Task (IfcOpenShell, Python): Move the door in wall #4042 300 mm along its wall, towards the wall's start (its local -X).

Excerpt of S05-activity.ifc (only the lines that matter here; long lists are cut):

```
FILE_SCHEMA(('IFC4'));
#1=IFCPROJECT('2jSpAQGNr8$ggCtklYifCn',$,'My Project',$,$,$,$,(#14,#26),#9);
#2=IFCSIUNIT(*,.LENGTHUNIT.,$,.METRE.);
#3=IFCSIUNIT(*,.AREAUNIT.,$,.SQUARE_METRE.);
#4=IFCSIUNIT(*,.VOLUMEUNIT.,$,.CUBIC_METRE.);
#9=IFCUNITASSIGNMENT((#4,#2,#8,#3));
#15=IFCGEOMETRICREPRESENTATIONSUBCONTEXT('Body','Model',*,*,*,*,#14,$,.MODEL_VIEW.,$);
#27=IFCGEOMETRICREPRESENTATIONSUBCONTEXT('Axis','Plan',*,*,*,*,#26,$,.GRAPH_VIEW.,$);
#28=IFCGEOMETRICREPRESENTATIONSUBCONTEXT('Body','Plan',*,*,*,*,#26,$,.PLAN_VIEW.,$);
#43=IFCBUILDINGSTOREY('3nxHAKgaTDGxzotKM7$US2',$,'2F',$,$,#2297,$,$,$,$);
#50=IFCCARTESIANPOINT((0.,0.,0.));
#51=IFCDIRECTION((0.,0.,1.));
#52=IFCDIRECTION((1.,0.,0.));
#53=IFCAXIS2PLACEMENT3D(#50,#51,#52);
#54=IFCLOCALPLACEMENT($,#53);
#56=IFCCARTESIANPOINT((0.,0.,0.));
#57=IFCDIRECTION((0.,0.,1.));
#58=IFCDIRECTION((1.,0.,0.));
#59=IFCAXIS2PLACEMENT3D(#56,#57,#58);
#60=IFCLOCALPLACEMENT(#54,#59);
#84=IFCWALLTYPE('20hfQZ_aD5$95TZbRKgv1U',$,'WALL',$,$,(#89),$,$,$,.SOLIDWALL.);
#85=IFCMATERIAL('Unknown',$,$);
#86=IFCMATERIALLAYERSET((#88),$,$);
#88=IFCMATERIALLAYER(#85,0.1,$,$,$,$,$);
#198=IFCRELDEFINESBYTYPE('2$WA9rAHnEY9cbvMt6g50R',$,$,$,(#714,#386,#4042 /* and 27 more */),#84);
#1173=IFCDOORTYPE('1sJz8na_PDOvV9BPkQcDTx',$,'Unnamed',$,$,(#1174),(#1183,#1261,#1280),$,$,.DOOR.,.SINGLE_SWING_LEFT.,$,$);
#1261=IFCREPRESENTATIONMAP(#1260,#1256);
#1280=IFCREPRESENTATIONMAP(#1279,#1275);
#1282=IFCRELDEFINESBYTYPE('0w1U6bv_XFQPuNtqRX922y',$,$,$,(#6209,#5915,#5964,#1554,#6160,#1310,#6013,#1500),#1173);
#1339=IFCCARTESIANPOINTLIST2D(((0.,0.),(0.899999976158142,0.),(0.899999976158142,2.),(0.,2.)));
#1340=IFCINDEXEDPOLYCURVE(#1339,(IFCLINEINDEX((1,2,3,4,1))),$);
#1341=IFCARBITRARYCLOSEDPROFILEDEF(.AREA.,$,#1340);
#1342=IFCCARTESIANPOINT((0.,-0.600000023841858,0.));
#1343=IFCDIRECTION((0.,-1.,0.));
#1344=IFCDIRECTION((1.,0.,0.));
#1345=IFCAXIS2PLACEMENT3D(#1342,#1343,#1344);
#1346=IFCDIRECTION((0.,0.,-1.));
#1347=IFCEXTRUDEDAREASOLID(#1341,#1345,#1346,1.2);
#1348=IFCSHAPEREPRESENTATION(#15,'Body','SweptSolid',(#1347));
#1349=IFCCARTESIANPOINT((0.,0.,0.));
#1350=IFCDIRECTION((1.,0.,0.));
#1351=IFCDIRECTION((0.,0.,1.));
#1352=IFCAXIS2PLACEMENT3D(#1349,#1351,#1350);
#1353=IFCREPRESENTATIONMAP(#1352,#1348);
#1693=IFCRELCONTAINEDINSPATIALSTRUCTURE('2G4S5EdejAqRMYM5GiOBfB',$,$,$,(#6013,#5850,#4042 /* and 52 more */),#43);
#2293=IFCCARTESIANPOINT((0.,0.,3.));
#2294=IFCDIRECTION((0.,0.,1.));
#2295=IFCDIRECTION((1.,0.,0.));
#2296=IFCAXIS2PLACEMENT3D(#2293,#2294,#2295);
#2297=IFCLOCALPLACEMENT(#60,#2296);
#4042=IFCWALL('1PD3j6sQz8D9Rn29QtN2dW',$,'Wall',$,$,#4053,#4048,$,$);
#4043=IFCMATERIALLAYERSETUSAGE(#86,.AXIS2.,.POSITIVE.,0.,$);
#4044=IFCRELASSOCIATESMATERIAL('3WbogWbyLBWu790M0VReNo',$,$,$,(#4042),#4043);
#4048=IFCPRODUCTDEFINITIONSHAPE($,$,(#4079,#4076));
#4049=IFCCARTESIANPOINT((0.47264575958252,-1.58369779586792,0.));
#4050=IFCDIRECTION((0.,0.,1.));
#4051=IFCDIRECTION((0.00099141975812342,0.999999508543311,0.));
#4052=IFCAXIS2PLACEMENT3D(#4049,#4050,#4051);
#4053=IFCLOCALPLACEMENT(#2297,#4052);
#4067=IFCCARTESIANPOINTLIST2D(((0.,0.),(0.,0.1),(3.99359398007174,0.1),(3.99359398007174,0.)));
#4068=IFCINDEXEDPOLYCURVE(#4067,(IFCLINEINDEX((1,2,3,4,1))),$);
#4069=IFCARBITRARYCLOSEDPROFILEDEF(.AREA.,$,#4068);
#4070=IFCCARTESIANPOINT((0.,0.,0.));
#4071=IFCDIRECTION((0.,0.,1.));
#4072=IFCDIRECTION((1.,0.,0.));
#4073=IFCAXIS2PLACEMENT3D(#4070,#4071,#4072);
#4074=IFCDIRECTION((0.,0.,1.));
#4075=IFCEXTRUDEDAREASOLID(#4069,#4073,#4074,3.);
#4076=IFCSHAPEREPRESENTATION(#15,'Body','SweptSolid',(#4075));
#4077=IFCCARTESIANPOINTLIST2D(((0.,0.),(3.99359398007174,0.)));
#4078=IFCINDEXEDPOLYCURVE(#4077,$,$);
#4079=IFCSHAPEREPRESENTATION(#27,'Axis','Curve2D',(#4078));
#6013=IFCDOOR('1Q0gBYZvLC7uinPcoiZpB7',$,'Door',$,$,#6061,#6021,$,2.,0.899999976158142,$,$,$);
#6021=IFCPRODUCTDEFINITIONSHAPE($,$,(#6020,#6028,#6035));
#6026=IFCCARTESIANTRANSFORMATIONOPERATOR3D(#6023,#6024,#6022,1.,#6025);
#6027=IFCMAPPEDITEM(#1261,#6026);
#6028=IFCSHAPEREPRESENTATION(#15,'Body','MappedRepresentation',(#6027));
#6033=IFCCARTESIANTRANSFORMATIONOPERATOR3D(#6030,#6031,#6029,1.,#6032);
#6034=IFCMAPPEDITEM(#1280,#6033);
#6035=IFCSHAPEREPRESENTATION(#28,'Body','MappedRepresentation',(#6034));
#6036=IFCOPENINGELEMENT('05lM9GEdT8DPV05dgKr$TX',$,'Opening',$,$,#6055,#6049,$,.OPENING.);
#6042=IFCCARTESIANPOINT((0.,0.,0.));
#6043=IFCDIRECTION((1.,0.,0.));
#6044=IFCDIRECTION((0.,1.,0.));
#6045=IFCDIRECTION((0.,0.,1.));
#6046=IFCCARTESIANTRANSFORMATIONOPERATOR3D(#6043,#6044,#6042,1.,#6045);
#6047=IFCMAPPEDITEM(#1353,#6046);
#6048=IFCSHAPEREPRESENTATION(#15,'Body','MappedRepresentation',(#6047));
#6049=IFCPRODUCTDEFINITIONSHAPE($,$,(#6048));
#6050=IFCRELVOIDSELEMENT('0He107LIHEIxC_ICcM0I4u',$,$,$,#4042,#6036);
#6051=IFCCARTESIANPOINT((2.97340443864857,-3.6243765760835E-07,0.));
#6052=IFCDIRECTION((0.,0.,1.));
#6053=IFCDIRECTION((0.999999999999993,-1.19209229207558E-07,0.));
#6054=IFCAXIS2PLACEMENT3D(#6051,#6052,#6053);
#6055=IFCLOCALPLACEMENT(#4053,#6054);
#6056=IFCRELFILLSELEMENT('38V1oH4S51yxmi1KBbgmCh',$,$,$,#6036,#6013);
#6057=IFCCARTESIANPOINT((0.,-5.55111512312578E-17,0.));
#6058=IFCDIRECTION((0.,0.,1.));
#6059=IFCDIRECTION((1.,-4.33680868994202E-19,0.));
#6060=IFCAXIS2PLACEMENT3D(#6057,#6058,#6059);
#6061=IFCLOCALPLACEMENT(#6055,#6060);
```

```python
import ifcopenshell
import ifcopenshell.api.geometry
import ifcopenshell.util.placement

model = ifcopenshell.open("S05-activity.ifc")

door = model.by_guid("1Q0gBYZvLC7uinPcoiZpB7")
opening = door.FillsVoids[0].RelatingOpeningElement
wall = opening.VoidsElements[0].RelatingBuildingElement

wall_matrix = ifcopenshell.util.placement.get_local_placement(wall.ObjectPlacement)
shift = wall_matrix[:3, 0] * -0.3
before = ifcopenshell.util.placement.get_local_placement(door.ObjectPlacement)[:3, 3].copy()

# The door is placed relative to its opening, so it follows when the opening moves.
matrix = ifcopenshell.util.placement.get_local_placement(opening.ObjectPlacement)
matrix[:3, 3] += shift
ifcopenshell.api.geometry.edit_object_placement(
    model, product=opening, matrix=matrix, is_si=False, should_transform_children=True
)

after = ifcopenshell.util.placement.get_local_placement(door.ObjectPlacement)[:3, 3]
print("door moved by", (after - before).round(3) + 0.0)

model.write("S05-activity_updated.ifc")
```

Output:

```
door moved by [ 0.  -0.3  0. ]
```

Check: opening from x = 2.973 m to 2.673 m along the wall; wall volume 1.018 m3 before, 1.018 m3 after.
